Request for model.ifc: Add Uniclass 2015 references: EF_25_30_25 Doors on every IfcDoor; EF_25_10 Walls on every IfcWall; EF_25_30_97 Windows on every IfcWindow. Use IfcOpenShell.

First a look at what the model holds.

```python
import ifcopenshell

model = ifcopenshell.open("model.ifc")
print(model.schema)
print("classifications:", [c.Name for c in model.by_type("IfcClassification")])
for ifc_class in ("IfcDoor", "IfcRoof", "IfcStair", "IfcWall", "IfcWindow"):
    print(ifc_class, len(model.by_type(ifc_class)))
```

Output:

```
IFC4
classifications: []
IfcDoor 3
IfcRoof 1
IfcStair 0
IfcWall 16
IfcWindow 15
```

```python
import ifcopenshell
import ifcopenshell.api.classification

model = ifcopenshell.open("model.ifc")

system = ifcopenshell.api.classification.add_classification(model, classification="Uniclass 2015")

codes = {
    "IfcDoor": ("EF_25_30_25", "Doors"),
    "IfcWall": ("EF_25_10", "Walls"),
    "IfcWindow": ("EF_25_30_97", "Windows"),
}
for ifc_class, (code, name) in codes.items():
    products = model.by_type(ifc_class)
    ifcopenshell.api.classification.add_reference(
        model, products=products, classification=system, identification=code, name=name
    )
    print(code, len(products))

model.write("model_updated.ifc")
```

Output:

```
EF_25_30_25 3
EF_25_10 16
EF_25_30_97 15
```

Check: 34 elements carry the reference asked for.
